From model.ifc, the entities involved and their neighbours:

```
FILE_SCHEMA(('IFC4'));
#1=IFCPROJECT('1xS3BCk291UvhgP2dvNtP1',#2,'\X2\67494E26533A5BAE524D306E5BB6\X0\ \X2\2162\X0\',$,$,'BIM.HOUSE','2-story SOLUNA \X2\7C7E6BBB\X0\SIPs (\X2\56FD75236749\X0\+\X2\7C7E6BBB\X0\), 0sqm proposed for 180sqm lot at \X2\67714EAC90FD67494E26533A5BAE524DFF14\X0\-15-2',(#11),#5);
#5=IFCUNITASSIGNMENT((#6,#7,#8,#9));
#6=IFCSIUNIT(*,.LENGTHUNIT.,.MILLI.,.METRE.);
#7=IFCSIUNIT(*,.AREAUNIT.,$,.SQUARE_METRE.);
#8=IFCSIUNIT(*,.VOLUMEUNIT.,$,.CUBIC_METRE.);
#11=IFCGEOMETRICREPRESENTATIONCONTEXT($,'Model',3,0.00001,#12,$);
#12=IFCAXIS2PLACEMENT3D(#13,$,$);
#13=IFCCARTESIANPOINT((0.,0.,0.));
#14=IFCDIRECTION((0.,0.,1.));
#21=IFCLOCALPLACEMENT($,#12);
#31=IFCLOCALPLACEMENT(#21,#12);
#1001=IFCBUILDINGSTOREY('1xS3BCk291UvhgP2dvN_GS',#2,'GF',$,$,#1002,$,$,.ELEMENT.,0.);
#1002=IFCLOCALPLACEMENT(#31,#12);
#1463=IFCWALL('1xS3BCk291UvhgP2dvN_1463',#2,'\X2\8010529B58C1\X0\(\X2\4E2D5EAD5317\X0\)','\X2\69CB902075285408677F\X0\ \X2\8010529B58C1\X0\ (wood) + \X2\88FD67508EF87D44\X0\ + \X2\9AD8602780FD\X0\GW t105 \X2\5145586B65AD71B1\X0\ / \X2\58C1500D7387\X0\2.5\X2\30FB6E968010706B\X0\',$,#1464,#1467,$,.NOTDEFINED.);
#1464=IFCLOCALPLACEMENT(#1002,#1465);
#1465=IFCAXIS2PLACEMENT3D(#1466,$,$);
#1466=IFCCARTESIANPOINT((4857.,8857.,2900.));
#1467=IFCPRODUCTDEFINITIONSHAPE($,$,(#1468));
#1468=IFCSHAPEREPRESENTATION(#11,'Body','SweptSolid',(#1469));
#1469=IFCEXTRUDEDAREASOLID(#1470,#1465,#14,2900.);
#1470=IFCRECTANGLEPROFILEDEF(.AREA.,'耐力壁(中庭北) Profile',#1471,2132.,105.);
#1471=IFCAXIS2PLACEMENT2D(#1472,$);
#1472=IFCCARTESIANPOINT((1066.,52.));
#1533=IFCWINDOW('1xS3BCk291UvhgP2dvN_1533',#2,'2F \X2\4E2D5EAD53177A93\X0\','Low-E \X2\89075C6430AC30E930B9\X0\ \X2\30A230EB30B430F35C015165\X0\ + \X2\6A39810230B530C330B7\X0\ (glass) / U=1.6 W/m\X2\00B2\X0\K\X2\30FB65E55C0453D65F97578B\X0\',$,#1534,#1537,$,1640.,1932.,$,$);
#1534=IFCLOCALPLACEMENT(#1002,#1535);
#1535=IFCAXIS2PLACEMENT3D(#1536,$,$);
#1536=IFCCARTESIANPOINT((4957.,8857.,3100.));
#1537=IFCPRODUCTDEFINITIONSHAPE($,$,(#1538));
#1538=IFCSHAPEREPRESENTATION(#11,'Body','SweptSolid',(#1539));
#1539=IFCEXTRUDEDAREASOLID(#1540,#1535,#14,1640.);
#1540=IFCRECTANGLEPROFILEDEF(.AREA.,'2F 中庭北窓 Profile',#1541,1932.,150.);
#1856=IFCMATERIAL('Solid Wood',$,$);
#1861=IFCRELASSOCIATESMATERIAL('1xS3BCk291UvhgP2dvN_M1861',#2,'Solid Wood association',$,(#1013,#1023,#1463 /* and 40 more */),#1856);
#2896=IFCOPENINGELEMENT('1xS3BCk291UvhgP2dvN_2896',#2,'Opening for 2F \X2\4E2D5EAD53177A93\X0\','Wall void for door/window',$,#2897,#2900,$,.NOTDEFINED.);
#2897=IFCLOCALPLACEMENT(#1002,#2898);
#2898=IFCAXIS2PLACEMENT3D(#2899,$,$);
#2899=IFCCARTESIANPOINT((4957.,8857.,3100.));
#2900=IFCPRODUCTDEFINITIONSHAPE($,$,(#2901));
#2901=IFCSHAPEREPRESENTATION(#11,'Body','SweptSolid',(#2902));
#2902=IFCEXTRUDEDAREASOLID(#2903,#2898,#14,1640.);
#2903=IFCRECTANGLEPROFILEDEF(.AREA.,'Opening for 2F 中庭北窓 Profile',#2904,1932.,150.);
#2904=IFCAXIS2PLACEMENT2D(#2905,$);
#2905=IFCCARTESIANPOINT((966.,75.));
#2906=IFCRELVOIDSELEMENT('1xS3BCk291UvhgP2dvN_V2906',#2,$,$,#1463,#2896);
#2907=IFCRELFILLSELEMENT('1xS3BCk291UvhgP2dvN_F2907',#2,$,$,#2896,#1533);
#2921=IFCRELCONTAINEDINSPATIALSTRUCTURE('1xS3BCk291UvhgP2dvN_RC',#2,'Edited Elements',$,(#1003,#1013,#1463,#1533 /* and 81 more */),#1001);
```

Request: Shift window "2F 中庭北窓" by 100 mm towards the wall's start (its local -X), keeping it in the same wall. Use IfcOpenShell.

```python
import ifcopenshell
import ifcopenshell.api.geometry
import ifcopenshell.util.placement

model = ifcopenshell.open("model.ifc")

window = model.by_id(1533)
opening = window.FillsVoids[0].RelatingOpeningElement
wall = opening.VoidsElements[0].RelatingBuildingElement

wall_matrix = ifcopenshell.util.placement.get_local_placement(wall.ObjectPlacement)
shift = wall_matrix[:3, 0] * -100.0
before = ifcopenshell.util.placement.get_local_placement(window.ObjectPlacement)[:3, 3].copy()

# The window is not placed relative to its opening, so move both.
for product in (opening, window):
    matrix = ifcopenshell.util.placement.get_local_placement(product.ObjectPlacement)
    matrix[:3, 3] += shift
    ifcopenshell.api.geometry.edit_object_placement(model, product=product, matrix=matrix, is_si=False)

after = ifcopenshell.util.placement.get_local_placement(window.ObjectPlacement)[:3, 3]
print("window moved by", (after - before).round(3) + 0.0)

model.write("model_updated.ifc")
```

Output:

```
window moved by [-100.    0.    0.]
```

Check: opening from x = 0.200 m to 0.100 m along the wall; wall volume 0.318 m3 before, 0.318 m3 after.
